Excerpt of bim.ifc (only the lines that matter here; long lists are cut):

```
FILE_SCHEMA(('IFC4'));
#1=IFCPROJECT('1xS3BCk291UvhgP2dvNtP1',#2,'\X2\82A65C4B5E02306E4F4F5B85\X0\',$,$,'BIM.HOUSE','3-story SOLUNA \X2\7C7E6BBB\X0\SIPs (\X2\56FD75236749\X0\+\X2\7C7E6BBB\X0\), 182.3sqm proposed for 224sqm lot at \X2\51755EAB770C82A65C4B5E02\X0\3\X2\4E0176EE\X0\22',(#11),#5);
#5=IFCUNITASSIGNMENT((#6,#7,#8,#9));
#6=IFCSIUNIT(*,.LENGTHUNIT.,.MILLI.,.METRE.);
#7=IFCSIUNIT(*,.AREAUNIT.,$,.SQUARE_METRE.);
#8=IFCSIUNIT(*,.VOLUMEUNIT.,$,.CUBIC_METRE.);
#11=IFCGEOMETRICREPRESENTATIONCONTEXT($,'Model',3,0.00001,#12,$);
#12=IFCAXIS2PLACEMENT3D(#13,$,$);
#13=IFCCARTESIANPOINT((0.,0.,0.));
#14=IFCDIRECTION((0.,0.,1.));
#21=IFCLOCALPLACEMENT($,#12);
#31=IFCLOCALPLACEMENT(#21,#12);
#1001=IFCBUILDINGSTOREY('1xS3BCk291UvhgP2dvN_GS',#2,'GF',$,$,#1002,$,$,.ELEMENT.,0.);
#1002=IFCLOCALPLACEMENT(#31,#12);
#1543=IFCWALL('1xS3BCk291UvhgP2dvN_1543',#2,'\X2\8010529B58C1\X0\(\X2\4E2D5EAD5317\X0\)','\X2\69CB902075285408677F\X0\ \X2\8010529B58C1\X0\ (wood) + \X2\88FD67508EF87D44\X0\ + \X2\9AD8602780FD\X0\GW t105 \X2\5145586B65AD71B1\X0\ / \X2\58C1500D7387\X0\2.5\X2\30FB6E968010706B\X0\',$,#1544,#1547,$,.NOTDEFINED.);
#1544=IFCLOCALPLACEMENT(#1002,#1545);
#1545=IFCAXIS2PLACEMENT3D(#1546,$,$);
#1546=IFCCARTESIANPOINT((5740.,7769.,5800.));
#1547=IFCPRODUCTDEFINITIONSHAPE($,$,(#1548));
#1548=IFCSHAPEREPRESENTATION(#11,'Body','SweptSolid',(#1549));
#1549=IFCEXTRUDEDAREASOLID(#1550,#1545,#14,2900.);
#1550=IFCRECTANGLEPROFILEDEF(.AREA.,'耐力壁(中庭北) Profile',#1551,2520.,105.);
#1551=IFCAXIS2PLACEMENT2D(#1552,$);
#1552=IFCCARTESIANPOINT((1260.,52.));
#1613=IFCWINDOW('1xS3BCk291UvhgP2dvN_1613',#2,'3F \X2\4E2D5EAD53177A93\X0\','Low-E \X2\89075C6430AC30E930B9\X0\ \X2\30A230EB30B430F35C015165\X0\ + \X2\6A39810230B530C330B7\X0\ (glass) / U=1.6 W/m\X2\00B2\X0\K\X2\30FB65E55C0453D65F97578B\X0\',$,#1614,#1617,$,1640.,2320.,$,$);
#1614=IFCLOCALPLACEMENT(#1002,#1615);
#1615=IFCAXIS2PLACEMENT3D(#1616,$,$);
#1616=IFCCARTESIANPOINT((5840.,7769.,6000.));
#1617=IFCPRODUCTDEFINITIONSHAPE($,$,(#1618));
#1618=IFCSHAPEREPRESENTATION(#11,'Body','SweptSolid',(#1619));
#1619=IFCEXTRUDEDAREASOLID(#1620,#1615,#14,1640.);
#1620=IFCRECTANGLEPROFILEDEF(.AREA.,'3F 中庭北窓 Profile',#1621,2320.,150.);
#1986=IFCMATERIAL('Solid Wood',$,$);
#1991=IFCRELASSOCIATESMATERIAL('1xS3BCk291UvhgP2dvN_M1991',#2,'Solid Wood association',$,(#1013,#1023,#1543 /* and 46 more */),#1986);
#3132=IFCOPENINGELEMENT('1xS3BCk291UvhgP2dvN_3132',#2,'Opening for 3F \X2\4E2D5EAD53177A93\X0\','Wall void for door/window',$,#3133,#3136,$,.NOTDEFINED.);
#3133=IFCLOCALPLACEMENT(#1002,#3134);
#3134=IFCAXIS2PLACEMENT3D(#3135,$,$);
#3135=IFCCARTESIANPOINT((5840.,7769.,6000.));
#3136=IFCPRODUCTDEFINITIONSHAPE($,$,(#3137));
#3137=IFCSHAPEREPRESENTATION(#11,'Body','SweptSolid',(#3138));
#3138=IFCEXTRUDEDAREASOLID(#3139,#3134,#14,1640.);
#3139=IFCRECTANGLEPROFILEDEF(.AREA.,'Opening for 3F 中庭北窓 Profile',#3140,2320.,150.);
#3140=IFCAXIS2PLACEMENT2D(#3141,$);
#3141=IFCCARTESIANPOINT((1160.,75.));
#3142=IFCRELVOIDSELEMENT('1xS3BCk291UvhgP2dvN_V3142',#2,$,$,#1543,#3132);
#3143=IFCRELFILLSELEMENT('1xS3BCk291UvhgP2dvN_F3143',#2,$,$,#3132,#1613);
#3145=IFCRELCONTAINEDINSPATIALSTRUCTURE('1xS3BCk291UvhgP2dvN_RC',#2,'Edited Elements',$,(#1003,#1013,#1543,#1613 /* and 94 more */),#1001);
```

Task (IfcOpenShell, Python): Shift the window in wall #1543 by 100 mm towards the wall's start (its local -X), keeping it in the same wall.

```python
import ifcopenshell
import ifcopenshell.api.geometry
import ifcopenshell.util.placement

model = ifcopenshell.open("bim.ifc")

window = model.by_id(1613)
opening = window.FillsVoids[0].RelatingOpeningElement
wall = opening.VoidsElements[0].RelatingBuildingElement

wall_matrix = ifcopenshell.util.placement.get_local_placement(wall.ObjectPlacement)
shift = wall_matrix[:3, 0] * -100.0
before = ifcopenshell.util.placement.get_local_placement(window.ObjectPlacement)[:3, 3].copy()

# The window is not placed relative to its opening, so move both.
for product in (opening, window):
    matrix = ifcopenshell.util.placement.get_local_placement(product.ObjectPlacement)
    matrix[:3, 3] += shift
    ifcopenshell.api.geometry.edit_object_placement(model, product=product, matrix=matrix, is_si=False)

after = ifcopenshell.util.placement.get_local_placement(window.ObjectPlacement)[:3, 3]
print("window moved by", (after - before).round(3) + 0.0)

model.write("bim-out.ifc")
```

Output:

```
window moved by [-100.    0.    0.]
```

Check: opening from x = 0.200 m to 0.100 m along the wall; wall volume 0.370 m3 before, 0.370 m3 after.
